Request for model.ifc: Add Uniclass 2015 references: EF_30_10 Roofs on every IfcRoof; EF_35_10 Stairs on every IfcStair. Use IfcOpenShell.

First a look at what the model holds.

```python
import ifcopenshell

model = ifcopenshell.open("model.ifc")
print(model.schema)
print("classifications:", [c.Name for c in model.by_type("IfcClassification")])
for ifc_class in ("IfcDoor", "IfcRoof", "IfcStair", "IfcWall", "IfcWindow"):
    print(ifc_class, len(model.by_type(ifc_class)))
```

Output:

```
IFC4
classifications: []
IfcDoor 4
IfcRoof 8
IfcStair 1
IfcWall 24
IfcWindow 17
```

```python
import ifcopenshell
import ifcopenshell.api.classification

model = ifcopenshell.open("model.ifc")

system = ifcopenshell.api.classification.add_classification(model, classification="Uniclass 2015")

codes = {
    "IfcRoof": ("EF_30_10", "Roofs"),
    "IfcStair": ("EF_35_10", "Stairs"),
}
for ifc_class, (code, name) in codes.items():
    products = model.by_type(ifc_class)
    ifcopenshell.api.classification.add_reference(
        model, products=products, classification=system, identification=code, name=name
    )
    print(code, len(products))

model.write("model_edited.ifc")
```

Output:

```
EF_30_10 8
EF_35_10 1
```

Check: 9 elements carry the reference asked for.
